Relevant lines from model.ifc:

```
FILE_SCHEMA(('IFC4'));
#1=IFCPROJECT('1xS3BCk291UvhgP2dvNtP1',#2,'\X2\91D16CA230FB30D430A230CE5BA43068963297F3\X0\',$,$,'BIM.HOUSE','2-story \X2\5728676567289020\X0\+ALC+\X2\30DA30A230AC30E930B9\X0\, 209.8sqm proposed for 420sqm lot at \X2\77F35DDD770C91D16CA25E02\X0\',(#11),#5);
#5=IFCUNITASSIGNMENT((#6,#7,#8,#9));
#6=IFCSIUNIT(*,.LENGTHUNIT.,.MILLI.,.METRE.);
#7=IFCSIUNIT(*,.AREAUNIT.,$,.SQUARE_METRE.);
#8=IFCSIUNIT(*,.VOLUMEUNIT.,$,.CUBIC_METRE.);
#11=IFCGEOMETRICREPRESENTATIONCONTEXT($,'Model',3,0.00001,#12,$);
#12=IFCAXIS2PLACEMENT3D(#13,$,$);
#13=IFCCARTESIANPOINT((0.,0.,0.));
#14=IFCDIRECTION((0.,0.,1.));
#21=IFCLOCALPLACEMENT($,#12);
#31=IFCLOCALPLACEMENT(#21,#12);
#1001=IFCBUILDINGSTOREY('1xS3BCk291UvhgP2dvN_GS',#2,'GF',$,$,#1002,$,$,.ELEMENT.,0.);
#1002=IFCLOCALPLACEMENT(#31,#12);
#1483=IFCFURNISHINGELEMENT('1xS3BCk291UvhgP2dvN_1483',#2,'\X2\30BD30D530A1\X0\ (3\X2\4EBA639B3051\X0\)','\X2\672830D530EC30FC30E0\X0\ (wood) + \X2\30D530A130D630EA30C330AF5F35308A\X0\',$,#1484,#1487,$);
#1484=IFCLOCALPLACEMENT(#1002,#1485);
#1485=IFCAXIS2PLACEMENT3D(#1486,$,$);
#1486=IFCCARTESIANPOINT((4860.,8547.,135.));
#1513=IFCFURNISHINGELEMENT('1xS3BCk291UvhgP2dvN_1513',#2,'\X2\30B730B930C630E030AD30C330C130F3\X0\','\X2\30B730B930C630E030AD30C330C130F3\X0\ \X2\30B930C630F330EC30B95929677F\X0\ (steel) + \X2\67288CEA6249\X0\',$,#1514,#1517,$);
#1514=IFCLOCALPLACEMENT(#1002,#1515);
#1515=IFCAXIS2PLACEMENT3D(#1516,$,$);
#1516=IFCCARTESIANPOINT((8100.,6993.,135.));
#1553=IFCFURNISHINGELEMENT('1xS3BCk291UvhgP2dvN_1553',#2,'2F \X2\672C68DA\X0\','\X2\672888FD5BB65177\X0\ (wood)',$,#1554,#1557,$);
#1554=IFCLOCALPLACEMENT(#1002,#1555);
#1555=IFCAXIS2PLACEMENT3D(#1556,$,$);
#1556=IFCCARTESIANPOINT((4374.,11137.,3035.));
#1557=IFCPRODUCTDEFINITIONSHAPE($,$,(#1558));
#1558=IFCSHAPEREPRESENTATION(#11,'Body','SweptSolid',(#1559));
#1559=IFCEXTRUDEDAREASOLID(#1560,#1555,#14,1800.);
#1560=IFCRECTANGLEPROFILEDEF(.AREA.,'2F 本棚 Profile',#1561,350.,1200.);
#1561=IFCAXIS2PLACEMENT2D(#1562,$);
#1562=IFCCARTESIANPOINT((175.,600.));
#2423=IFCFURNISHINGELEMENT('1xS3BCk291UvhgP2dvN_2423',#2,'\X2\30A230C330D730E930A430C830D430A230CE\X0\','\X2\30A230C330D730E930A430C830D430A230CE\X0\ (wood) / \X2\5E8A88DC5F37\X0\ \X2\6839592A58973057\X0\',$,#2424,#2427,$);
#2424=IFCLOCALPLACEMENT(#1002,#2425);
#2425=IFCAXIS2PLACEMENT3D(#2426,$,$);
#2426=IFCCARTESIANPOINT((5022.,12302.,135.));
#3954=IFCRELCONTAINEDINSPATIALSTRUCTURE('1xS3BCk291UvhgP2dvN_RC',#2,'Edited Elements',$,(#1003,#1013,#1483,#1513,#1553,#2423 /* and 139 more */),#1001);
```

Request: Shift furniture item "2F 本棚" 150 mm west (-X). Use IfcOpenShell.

```python
import ifcopenshell
import ifcopenshell.api.geometry
import ifcopenshell.util.placement
import ifcopenshell.util.unit

model = ifcopenshell.open("model.ifc")
unit_scale = ifcopenshell.util.unit.calculate_unit_scale(model)

item = model.by_id(1553)
matrix = ifcopenshell.util.placement.get_local_placement(item.ObjectPlacement)
matrix[0, 3] -= 0.15 / unit_scale
ifcopenshell.api.geometry.edit_object_placement(model, product=item, matrix=matrix, is_si=False)

print(ifcopenshell.util.placement.get_local_placement(item.ObjectPlacement).round(3) + 0.0)

model.write("model_v2.ifc")
```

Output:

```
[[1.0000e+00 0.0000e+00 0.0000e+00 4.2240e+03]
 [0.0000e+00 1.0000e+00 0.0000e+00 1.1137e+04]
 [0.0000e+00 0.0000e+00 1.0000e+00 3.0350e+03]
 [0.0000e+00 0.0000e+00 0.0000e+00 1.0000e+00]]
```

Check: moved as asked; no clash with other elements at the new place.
